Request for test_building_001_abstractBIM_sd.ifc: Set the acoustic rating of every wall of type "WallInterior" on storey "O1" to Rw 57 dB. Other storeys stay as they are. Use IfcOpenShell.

First a look at what the model holds.

```python
import ifcopenshell
import ifcopenshell.util.element

model = ifcopenshell.open("test_building_001_abstractBIM_sd.ifc")
print(model.schema)
storey = next(s for s in model.by_type("IfcBuildingStorey") if s.Name == "O1")
walls = [e for e in ifcopenshell.util.element.get_decomposition(storey) if e.is_a("IfcWall")]
seen = {}
for e in walls:
    element_type = ifcopenshell.util.element.get_type(e)
    key = (element_type.Name if element_type != e and element_type else None, ifcopenshell.util.element.get_pset(e, "Pset_WallCommon", "AcousticRating"))
    seen[key] = seen.get(key, 0) + 1
for (name, value), count in sorted(seen.items(), key=str):
    print(count, "x", name, "|", value)
```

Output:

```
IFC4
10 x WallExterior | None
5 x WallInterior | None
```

```python
import ifcopenshell
import ifcopenshell.api.pset
import ifcopenshell.util.element

model = ifcopenshell.open("test_building_001_abstractBIM_sd.ifc")

storey = next(s for s in model.by_type("IfcBuildingStorey") if s.Name == "O1")
walls = [e for e in ifcopenshell.util.element.get_decomposition(storey) if e.is_a("IfcWall")]

count = 0
for e in walls:
    element_type = ifcopenshell.util.element.get_type(e)
    if element_type in (None, e) or element_type.Name != "WallInterior":
        continue
    # add_pset returns the element's existing set when there is one.
    pset = ifcopenshell.api.pset.add_pset(model, product=e, name="Pset_WallCommon")
    ifcopenshell.api.pset.edit_pset(model, pset=pset, properties={"AcousticRating": "Rw 57 dB"})
    count += 1

print(count, "walls updated")

model.write("test_building_001_abstractBIM_sd_updated.ifc")
```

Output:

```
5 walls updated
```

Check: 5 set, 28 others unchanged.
